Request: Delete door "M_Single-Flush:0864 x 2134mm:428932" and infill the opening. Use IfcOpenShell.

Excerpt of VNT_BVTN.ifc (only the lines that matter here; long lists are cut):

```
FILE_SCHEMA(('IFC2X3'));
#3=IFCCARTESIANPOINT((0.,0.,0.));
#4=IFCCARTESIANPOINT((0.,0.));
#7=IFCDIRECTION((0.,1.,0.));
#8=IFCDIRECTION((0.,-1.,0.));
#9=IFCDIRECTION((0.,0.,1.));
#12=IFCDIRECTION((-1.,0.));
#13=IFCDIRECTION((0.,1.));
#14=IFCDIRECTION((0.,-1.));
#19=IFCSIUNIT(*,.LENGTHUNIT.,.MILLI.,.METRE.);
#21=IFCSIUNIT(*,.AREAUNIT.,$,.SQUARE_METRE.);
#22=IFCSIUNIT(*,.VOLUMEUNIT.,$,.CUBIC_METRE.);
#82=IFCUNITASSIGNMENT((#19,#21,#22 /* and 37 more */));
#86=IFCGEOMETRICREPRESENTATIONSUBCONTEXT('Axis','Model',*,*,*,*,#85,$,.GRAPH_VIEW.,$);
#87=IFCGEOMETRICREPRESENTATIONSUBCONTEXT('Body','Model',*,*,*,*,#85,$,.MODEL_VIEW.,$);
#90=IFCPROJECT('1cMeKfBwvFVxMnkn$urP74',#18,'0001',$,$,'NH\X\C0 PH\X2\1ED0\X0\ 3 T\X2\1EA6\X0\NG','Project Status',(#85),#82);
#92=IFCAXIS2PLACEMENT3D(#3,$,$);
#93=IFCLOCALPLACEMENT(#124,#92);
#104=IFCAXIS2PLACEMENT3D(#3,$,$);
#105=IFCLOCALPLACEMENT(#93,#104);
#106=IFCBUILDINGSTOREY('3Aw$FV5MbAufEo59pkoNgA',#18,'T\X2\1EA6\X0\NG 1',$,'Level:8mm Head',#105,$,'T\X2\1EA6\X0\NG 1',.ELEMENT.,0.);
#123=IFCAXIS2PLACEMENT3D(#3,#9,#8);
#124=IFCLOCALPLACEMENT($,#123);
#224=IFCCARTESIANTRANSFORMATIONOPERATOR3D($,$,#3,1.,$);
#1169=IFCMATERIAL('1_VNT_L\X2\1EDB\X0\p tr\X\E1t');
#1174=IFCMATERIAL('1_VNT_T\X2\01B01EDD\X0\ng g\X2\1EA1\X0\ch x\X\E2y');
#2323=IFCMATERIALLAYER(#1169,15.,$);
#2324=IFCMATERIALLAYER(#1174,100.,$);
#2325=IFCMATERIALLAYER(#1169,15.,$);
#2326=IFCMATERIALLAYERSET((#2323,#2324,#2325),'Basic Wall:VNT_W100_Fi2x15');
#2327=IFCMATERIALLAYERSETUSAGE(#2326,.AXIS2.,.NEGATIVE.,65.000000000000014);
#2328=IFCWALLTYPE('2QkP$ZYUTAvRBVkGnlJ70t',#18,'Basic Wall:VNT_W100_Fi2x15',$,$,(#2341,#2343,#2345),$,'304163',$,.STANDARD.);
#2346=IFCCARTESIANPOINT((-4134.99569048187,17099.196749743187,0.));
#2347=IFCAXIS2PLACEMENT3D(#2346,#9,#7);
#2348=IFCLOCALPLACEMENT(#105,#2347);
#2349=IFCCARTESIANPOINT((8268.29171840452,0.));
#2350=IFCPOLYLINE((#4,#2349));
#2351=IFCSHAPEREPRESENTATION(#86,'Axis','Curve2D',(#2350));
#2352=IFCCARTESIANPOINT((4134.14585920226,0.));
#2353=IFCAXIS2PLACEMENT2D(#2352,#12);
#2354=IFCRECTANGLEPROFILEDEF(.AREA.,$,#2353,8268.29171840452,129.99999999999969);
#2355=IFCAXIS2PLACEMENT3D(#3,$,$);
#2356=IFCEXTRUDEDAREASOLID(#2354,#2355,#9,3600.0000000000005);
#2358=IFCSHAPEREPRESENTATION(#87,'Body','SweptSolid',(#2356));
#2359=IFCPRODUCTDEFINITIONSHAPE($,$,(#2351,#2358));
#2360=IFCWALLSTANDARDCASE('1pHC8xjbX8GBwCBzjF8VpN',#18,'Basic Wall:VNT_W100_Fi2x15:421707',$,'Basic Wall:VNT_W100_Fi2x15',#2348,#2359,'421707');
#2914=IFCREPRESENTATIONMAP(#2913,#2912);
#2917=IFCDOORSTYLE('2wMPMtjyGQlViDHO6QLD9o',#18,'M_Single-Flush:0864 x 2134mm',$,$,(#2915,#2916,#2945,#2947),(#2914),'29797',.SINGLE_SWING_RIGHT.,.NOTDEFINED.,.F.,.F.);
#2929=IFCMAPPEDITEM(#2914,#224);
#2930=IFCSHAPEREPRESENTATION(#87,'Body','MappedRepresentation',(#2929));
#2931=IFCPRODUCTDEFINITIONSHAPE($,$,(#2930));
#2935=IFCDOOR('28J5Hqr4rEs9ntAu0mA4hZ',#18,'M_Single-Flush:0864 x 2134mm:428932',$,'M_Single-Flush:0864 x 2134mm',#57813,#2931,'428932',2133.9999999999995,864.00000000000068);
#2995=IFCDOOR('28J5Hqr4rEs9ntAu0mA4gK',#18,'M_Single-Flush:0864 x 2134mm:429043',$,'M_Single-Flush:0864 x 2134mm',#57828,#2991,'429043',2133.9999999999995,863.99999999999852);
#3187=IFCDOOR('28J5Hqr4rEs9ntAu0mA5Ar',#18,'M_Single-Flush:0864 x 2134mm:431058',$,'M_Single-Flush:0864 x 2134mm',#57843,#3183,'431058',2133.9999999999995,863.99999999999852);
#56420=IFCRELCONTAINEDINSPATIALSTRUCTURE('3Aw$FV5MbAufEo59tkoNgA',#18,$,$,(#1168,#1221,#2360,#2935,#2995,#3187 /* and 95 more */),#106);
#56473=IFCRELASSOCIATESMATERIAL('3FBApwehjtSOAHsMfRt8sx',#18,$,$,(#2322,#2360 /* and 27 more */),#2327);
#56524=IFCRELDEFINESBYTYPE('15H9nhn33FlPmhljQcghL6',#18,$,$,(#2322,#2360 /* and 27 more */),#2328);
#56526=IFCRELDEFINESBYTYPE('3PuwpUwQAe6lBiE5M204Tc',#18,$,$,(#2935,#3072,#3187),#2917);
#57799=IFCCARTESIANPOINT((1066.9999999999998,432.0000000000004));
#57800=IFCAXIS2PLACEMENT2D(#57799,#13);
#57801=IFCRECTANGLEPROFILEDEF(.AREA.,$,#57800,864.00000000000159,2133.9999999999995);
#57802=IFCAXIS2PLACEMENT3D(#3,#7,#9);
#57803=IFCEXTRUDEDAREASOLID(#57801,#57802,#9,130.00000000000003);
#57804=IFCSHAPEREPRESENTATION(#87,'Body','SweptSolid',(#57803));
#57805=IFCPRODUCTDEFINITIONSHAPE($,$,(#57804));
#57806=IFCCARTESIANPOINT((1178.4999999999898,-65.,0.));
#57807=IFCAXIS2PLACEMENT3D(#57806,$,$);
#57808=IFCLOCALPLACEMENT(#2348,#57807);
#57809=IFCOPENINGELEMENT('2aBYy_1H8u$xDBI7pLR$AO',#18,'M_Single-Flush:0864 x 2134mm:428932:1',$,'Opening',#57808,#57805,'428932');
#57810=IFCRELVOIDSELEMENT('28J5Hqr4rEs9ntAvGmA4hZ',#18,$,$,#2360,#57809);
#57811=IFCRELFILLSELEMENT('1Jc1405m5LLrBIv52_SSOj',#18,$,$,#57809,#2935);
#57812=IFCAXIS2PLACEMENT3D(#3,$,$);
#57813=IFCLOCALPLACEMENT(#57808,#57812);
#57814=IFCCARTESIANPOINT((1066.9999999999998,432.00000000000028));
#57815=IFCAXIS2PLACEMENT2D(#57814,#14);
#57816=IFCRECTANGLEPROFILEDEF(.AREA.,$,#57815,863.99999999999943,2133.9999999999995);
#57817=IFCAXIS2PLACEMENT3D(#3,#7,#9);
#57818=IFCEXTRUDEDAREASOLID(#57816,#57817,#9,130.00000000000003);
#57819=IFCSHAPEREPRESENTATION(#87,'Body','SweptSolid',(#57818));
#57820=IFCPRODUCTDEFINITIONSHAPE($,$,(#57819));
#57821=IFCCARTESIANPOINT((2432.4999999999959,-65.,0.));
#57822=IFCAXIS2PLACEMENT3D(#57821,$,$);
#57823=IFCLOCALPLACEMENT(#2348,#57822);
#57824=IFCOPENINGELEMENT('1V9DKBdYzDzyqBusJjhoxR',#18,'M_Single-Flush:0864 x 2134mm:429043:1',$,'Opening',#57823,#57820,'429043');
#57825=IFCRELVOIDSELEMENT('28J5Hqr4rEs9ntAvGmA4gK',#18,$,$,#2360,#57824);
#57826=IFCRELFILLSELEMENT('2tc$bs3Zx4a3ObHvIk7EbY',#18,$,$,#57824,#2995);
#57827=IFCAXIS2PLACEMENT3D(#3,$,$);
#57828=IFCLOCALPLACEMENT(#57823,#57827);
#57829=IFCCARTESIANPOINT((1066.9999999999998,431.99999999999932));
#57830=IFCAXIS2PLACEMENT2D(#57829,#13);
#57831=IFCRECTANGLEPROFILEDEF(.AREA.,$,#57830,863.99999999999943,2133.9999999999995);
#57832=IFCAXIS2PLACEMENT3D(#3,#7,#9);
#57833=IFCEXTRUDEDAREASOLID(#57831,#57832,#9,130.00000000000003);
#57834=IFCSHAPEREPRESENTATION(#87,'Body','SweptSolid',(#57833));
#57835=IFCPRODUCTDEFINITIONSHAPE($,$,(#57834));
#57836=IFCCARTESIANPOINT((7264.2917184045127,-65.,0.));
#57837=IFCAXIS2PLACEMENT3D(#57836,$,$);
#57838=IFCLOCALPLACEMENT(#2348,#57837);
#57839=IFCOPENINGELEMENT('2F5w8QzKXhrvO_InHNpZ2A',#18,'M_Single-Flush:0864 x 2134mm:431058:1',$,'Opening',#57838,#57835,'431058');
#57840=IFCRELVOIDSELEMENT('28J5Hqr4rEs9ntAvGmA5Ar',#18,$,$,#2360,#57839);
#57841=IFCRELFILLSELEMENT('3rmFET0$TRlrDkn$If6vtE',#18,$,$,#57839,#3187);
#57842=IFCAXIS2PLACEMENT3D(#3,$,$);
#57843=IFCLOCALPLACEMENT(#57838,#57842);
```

```python
import ifcopenshell
import ifcopenshell.api.feature
import ifcopenshell.api.root
import ifcopenshell.geom
import ifcopenshell.util.shape

model = ifcopenshell.open("VNT_BVTN.ifc")
settings = ifcopenshell.geom.settings()


def volume(element):
    """Net volume in cubic metres, openings subtracted."""
    shape = ifcopenshell.geom.create_shape(settings, element)
    return ifcopenshell.util.shape.get_volume(shape.geometry)


door = model.by_guid("28J5Hqr4rEs9ntAu0mA4hZ")
opening = door.FillsVoids[0].RelatingOpeningElement
wall = opening.VoidsElements[0].RelatingBuildingElement
before = volume(wall)

ifcopenshell.api.root.remove_product(model, product=door)
ifcopenshell.api.feature.remove_feature(model, feature=opening)

after = volume(wall)

print(f"wall volume {before:.3f} -> {after:.3f} m3")

model.write("VNT_BVTN_rev.ifc")
```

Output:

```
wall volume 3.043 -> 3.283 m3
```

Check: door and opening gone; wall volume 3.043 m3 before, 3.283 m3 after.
